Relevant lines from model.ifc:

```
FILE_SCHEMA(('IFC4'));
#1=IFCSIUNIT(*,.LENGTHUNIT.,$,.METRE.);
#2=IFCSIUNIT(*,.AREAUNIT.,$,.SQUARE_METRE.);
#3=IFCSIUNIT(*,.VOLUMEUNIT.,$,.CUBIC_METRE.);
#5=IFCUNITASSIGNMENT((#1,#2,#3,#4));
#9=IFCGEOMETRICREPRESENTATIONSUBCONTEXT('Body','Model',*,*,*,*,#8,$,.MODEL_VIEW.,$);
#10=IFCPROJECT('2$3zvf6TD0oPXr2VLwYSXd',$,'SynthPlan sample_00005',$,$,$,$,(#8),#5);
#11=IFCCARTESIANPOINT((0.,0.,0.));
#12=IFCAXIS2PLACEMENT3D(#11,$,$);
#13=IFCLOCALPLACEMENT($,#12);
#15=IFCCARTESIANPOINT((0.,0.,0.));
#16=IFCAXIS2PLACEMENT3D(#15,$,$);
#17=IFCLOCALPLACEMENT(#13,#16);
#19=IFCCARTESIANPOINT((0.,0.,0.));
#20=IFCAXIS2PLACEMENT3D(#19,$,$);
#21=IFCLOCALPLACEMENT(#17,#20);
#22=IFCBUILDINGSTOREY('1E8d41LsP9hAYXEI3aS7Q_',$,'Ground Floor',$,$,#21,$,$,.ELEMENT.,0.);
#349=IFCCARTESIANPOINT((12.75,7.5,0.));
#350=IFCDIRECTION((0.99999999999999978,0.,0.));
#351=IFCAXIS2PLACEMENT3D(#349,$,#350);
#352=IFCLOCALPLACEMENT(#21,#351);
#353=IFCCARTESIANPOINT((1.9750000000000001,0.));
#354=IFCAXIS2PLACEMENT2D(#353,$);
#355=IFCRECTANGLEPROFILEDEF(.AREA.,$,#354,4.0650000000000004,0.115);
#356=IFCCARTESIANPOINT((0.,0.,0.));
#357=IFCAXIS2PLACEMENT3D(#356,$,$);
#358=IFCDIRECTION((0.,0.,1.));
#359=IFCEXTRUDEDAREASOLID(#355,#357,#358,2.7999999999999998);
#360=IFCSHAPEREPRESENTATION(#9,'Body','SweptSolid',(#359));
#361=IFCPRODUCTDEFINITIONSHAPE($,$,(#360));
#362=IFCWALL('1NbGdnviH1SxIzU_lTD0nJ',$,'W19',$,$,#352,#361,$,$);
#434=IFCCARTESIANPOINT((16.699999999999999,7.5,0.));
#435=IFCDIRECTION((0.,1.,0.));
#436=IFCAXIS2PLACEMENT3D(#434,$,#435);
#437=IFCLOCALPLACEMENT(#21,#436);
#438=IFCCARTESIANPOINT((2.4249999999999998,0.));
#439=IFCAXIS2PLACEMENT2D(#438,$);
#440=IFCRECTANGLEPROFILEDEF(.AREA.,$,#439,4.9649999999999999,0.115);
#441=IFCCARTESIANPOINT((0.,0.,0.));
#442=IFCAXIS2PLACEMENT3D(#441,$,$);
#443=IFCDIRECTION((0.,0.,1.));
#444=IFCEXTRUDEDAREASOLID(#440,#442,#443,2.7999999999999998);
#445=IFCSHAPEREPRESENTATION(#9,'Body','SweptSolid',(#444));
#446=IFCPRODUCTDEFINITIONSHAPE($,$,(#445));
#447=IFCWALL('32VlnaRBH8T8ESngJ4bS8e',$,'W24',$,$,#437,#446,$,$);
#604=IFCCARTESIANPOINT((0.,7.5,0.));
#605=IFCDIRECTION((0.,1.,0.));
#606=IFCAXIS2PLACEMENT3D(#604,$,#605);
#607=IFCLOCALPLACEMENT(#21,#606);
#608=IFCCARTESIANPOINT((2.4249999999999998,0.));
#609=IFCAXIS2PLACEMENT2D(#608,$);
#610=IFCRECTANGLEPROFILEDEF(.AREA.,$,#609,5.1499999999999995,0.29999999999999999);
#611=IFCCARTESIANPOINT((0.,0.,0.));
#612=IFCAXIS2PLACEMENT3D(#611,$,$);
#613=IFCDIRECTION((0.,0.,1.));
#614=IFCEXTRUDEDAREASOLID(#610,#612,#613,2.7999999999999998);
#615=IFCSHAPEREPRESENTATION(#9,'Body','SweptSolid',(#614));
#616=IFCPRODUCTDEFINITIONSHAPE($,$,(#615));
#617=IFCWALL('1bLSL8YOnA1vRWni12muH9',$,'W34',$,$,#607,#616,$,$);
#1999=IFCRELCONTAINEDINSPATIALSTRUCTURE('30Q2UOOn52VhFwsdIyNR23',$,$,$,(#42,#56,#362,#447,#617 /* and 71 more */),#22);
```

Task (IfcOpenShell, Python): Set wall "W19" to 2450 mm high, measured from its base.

```python
import ifcopenshell
import ifcopenshell.geom
import ifcopenshell.util.representation
import ifcopenshell.util.shape
import ifcopenshell.util.unit

model = ifcopenshell.open("model.ifc")
unit_scale = ifcopenshell.util.unit.calculate_unit_scale(model)
settings = ifcopenshell.geom.settings()


def volume(element):
    """Net volume in cubic metres, openings subtracted."""
    shape = ifcopenshell.geom.create_shape(settings, element)
    return ifcopenshell.util.shape.get_volume(shape.geometry)


wall = model.by_guid("1NbGdnviH1SxIzU_lTD0nJ")
before = volume(wall)

body = ifcopenshell.util.representation.get_representation(wall, "Model", "Body")
solid = body.Items[0]
old_height = solid.Depth
solid.Depth = 2.45 / unit_scale
after = volume(wall)

print(f"height {old_height:g} -> {solid.Depth:g}, volume {before:.3f} -> {after:.3f} m3")

model.write("model_edited.ifc")
```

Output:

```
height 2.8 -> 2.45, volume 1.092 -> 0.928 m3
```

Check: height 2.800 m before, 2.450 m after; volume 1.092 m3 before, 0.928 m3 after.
